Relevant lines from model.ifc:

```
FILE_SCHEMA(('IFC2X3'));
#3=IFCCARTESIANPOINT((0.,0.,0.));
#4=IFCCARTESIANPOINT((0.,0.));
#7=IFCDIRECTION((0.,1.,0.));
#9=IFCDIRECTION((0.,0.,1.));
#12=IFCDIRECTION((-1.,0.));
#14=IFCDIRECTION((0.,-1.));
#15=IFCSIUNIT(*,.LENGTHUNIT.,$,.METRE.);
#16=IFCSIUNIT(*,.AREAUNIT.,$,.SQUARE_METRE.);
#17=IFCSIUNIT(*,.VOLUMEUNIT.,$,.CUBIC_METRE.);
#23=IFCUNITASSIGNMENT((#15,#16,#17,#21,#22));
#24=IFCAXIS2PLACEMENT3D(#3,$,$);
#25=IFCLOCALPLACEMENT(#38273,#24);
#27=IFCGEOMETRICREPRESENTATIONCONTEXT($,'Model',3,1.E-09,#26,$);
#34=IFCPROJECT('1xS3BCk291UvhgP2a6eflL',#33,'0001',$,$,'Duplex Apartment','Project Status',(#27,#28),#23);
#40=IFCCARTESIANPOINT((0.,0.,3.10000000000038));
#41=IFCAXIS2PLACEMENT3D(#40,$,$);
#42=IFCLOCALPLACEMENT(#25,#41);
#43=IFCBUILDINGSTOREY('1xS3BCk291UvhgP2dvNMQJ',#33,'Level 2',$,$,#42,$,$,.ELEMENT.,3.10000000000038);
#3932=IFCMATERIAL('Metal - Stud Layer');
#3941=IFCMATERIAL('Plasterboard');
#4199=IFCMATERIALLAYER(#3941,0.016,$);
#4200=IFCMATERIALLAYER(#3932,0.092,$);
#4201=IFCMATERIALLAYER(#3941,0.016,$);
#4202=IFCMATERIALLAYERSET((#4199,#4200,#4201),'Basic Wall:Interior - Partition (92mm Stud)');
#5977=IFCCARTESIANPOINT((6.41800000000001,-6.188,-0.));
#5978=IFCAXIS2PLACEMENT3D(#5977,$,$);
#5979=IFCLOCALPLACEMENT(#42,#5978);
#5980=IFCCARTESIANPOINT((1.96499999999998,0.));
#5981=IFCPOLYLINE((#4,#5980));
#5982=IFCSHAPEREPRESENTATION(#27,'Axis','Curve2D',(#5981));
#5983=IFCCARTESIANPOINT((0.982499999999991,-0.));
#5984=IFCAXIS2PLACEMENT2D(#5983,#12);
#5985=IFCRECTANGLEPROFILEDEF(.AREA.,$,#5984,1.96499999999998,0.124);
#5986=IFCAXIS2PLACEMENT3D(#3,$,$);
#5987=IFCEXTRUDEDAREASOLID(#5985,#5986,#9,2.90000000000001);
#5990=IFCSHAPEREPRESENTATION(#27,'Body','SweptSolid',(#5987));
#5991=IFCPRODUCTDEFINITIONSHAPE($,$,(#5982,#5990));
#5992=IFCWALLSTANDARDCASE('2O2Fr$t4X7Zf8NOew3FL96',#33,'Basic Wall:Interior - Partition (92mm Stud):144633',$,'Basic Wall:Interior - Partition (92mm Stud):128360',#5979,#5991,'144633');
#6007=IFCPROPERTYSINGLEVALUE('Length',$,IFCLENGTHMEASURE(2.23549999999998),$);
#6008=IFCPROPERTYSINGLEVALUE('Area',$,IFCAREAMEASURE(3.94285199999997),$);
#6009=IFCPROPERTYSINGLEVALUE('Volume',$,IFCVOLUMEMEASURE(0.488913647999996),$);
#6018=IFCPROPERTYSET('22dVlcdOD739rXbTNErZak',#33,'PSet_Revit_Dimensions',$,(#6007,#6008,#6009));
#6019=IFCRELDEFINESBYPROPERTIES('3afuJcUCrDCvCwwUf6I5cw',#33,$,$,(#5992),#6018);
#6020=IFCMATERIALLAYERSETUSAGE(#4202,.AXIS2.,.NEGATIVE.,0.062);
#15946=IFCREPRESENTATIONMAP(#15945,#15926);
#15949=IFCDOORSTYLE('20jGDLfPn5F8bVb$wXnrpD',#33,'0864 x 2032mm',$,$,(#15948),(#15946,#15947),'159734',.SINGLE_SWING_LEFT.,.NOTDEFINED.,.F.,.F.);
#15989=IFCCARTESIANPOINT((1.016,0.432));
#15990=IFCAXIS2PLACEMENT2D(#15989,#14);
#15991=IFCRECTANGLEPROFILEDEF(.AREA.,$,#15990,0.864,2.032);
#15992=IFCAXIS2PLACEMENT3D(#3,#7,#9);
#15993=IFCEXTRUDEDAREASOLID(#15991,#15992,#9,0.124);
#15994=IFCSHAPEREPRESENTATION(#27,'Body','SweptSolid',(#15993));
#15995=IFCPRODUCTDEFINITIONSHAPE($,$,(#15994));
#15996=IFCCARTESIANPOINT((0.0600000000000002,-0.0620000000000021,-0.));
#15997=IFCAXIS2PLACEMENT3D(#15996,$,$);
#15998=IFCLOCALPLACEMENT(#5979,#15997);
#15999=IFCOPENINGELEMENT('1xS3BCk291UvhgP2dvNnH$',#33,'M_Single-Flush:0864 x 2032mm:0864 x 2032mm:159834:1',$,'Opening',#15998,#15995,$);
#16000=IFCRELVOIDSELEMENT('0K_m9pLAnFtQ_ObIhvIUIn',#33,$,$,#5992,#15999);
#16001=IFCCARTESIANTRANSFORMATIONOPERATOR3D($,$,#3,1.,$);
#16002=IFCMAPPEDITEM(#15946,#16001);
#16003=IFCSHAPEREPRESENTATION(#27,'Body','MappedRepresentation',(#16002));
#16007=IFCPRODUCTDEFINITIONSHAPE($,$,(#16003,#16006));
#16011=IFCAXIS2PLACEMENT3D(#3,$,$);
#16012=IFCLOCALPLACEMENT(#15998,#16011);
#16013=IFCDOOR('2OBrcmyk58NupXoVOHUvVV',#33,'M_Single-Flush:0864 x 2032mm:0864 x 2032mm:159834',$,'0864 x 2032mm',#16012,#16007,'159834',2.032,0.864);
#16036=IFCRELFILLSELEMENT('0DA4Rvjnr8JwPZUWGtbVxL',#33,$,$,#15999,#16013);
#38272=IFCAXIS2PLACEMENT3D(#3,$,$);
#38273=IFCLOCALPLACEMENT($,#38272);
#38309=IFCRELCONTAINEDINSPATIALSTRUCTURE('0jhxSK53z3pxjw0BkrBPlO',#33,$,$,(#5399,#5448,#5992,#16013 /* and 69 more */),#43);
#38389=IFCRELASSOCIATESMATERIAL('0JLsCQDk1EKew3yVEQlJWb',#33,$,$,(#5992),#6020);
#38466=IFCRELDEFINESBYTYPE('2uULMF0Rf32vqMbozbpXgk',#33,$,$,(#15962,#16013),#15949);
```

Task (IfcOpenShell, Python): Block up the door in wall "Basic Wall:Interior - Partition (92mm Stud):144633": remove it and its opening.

```python
import ifcopenshell
import ifcopenshell.api.feature
import ifcopenshell.api.pset
import ifcopenshell.api.root
import ifcopenshell.geom
import ifcopenshell.util.element
import ifcopenshell.util.shape
import ifcopenshell.util.unit

model = ifcopenshell.open("model.ifc")
area_scale = ifcopenshell.util.unit.calculate_unit_scale(model, "AREAUNIT")
volume_scale = ifcopenshell.util.unit.calculate_unit_scale(model, "VOLUMEUNIT")
settings = ifcopenshell.geom.settings()


def volume(element):
    """Net volume in cubic metres, openings subtracted."""
    shape = ifcopenshell.geom.create_shape(settings, element)
    return ifcopenshell.util.shape.get_volume(shape.geometry)


door = model.by_guid("2OBrcmyk58NupXoVOHUvVV")
opening = door.FillsVoids[0].RelatingOpeningElement
wall = opening.VoidsElements[0].RelatingBuildingElement
before = volume(wall)

ifcopenshell.api.root.remove_product(model, product=door)
ifcopenshell.api.feature.remove_feature(model, feature=opening)

after = volume(wall)
thickness = 0.124  # wall thickness in metres

# Update the wall's stored quantities.
pset = model.by_id(ifcopenshell.util.element.get_pset(wall, "PSet_Revit_Dimensions", should_inherit=False)["id"])
ifcopenshell.api.pset.edit_pset(model, pset=pset, properties={
    "Area": model.create_entity("IfcAreaMeasure", after / thickness / area_scale),
    "Volume": model.create_entity("IfcVolumeMeasure", after / volume_scale),
})

print(f"wall volume {before:.3f} -> {after:.3f} m3")

model.write("model_updated.ifc")
```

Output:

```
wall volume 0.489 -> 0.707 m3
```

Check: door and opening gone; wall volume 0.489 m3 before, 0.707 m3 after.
